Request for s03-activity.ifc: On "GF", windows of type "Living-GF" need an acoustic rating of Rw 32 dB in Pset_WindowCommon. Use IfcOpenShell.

First a look at what the model holds.

```python
import ifcopenshell
import ifcopenshell.util.element

model = ifcopenshell.open("s03-activity.ifc")
print(model.schema)
storey = next(s for s in model.by_type("IfcBuildingStorey") if s.Name == "GF")
windows = [e for e in ifcopenshell.util.element.get_decomposition(storey) if e.is_a("IfcWindow")]
seen = {}
for e in windows:
    element_type = ifcopenshell.util.element.get_type(e)
    key = (element_type.Name if element_type != e and element_type else None, ifcopenshell.util.element.get_pset(e, "Pset_WindowCommon", "AcousticRating"))
    seen[key] = seen.get(key, 0) + 1
for (name, value), count in sorted(seen.items(), key=str):
    print(count, "x", name, "|", value)
```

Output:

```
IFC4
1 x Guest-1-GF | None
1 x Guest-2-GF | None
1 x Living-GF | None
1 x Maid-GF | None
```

```python
import ifcopenshell
import ifcopenshell.api.pset
import ifcopenshell.util.element

model = ifcopenshell.open("s03-activity.ifc")

storey = next(s for s in model.by_type("IfcBuildingStorey") if s.Name == "GF")
windows = [e for e in ifcopenshell.util.element.get_decomposition(storey) if e.is_a("IfcWindow")]

count = 0
for e in windows:
    element_type = ifcopenshell.util.element.get_type(e)
    if element_type in (None, e) or element_type.Name != "Living-GF":
        continue
    # add_pset returns the element's existing set when there is one.
    pset = ifcopenshell.api.pset.add_pset(model, product=e, name="Pset_WindowCommon")
    ifcopenshell.api.pset.edit_pset(model, pset=pset, properties={"AcousticRating": "Rw 32 dB"})
    count += 1

print(count, "windows updated")

model.write("s03-activity-out.ifc")
```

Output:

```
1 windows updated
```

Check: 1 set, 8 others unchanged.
